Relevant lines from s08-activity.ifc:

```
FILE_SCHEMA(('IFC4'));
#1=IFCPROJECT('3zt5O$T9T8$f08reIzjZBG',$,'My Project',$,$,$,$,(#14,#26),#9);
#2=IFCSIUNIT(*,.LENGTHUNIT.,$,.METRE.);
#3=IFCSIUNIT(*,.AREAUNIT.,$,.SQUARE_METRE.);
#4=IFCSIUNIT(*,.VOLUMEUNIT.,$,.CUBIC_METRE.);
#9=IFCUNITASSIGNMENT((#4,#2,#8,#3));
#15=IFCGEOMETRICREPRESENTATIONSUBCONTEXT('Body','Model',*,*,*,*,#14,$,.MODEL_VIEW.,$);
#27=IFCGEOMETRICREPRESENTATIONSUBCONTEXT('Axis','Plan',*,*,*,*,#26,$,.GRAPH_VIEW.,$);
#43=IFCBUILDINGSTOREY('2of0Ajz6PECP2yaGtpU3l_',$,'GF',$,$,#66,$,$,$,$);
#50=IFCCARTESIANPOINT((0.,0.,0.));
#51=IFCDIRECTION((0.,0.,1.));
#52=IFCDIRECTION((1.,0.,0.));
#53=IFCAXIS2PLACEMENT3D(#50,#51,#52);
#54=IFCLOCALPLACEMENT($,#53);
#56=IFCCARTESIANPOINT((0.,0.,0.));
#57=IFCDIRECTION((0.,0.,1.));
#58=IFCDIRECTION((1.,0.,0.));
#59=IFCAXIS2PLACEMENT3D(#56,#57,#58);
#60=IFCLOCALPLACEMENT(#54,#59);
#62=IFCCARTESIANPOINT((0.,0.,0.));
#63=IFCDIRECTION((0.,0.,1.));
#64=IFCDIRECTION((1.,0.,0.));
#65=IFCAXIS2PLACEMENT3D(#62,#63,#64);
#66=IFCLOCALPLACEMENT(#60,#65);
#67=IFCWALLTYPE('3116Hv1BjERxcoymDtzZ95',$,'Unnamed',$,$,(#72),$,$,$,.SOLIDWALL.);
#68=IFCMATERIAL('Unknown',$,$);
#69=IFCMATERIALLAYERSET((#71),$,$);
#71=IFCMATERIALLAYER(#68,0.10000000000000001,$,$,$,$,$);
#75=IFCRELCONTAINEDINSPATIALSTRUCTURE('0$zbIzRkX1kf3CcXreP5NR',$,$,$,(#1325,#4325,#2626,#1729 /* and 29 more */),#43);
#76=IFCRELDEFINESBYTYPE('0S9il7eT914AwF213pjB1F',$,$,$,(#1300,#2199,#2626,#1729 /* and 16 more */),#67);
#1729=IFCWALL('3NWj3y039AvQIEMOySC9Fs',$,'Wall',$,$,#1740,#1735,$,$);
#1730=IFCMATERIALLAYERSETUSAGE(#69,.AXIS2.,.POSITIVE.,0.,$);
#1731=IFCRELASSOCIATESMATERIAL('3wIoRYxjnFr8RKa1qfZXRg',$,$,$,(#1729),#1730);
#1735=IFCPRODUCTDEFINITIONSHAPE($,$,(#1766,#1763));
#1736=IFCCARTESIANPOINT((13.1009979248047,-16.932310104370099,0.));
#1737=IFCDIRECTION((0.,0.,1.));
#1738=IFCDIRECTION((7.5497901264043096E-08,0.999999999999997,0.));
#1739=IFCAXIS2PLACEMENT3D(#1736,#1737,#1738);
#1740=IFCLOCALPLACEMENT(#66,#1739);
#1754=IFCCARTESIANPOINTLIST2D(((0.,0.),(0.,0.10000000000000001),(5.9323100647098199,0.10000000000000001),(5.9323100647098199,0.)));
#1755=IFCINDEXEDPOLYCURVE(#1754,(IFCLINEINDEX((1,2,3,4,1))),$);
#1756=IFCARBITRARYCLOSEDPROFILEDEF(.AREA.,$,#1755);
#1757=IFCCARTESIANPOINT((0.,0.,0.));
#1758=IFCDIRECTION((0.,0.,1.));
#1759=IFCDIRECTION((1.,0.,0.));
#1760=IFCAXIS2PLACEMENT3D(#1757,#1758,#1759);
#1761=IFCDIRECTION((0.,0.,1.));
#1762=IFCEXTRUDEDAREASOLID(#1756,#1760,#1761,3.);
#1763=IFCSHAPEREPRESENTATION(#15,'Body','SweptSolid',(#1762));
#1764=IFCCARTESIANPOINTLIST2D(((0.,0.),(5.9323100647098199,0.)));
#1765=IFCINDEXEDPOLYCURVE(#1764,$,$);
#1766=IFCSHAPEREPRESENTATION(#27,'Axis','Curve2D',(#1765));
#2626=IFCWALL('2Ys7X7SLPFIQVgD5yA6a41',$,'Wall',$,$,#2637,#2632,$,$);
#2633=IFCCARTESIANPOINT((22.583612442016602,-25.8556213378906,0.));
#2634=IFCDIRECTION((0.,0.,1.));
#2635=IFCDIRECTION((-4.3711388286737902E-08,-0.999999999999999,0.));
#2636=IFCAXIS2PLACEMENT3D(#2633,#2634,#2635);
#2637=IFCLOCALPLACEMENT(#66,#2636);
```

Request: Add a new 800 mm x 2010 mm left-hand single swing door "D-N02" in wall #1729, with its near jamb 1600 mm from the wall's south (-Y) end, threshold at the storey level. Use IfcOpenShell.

```python
import numpy as np
import ifcopenshell
import ifcopenshell.api.feature
import ifcopenshell.api.geometry
import ifcopenshell.api.root
import ifcopenshell.api.spatial
import ifcopenshell.geom
import ifcopenshell.util.element
import ifcopenshell.util.placement
import ifcopenshell.util.representation
import ifcopenshell.util.shape
import ifcopenshell.util.unit

model = ifcopenshell.open("s08-activity.ifc")
unit_scale = ifcopenshell.util.unit.calculate_unit_scale(model)
settings = ifcopenshell.geom.settings()


def volume(element):
    """Net volume in cubic metres, openings subtracted."""
    shape = ifcopenshell.geom.create_shape(settings, element)
    return ifcopenshell.util.shape.get_volume(shape.geometry)


wall = model.by_guid("3NWj3y039AvQIEMOySC9Fs")
storey = ifcopenshell.util.element.get_container(wall, ifc_class="IfcBuildingStorey")
context = ifcopenshell.util.representation.get_context(model, "Model", "Body", "MODEL_VIEW")
before = volume(wall)

width, height, from_end, sill = 0.8, 2.01, 1.6, 0.0  # metres

# The wall runs along its own X axis, and the end named is its -X end.
wall_shape = ifcopenshell.geom.create_shape(settings, wall)
x, y, z = ifcopenshell.util.shape.get_vertices(wall_shape.geometry).T
start = x.min() + from_end
face, thickness = float(y.min()), float(y.max() - y.min())
wall_matrix = ifcopenshell.util.placement.get_local_placement(wall.ObjectPlacement)
level = ifcopenshell.util.placement.get_local_placement(storey.ObjectPlacement)[2, 3]


def in_wall(x, y):
    """Placement at x, y metres in the wall's axes, at sill height."""
    matrix = wall_matrix.copy()
    matrix[:, 3] = wall_matrix @ np.array([x / unit_scale, y / unit_scale, 0.0, 1.0])
    matrix[2, 3] = level + sill / unit_scale
    return matrix


# Opening: a box that overshoots both wall faces by 50 mm.
opening = ifcopenshell.api.root.create_entity(model, ifc_class="IfcOpeningElement", predefined_type="OPENING")
box = ifcopenshell.api.geometry.add_wall_representation(
    model, context=context, length=width, height=height, thickness=thickness + 0.1
)
ifcopenshell.api.geometry.assign_representation(model, product=opening, representation=box)
ifcopenshell.api.geometry.edit_object_placement(model, product=opening, matrix=in_wall(start, face - 0.05), is_si=False)
ifcopenshell.api.feature.add_feature(model, feature=opening, element=wall)

door = ifcopenshell.api.root.create_entity(model, ifc_class="IfcDoor", name="D-N02", predefined_type="DOOR")
door.OverallWidth, door.OverallHeight = width / unit_scale, height / unit_scale
door.OperationType = "SINGLE_SWING_LEFT"
body = ifcopenshell.api.geometry.add_door_representation(
    model,
    context=context,
    overall_width=door.OverallWidth,
    overall_height=door.OverallHeight,
    operation_type="SINGLE_SWING_LEFT",
    lining_properties={"LiningDepth": thickness / unit_scale, "ThresholdDepth": thickness / unit_scale},
)
ifcopenshell.api.geometry.assign_representation(model, product=door, representation=body)
ifcopenshell.api.spatial.assign_container(model, products=[door], relating_structure=storey)
ifcopenshell.api.feature.add_filling(model, opening=opening, element=door)

# The lining spans the wall, so the door starts at the wall face.
ifcopenshell.api.geometry.edit_object_placement(model, product=door, matrix=in_wall(start, face), is_si=False)

after = volume(wall)

print(f"wall volume {before:.3f} -> {after:.3f} m3")

model.write("s08-activity-out.ifc")
```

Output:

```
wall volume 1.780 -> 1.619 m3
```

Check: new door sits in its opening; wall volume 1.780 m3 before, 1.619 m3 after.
